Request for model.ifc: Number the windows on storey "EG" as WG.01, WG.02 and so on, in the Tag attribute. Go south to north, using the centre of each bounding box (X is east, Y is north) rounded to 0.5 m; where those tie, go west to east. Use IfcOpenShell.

First a look at what the model holds.

```python
import ifcopenshell
import ifcopenshell.util.element
import ifcopenshell.util.placement

model = ifcopenshell.open("model.ifc")
print(model.schema)
storey = next(s for s in model.by_type("IfcBuildingStorey") if s.Name == "EG")
windows = [e for e in ifcopenshell.util.element.get_decomposition(storey) if e.is_a("IfcWindow")]
for e in sorted(windows, key=lambda e: e.id()):
    origin = ifcopenshell.util.placement.get_local_placement(e.ObjectPlacement)[:3, 3]
    print(e.id(), e.Tag, e.Name, origin.round(2) + 0.0, sep=" | ")
```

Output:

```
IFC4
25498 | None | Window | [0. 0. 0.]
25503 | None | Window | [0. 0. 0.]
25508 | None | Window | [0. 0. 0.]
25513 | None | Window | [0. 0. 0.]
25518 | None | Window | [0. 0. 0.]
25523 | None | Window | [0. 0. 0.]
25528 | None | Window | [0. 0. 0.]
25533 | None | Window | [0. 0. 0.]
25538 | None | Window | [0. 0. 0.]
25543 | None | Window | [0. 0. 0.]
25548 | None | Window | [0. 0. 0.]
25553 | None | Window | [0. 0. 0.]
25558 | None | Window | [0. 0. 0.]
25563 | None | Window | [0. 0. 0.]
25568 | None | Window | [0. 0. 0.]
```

```python
import ifcopenshell
import ifcopenshell.geom
import ifcopenshell.util.element
import ifcopenshell.util.shape

model = ifcopenshell.open("model.ifc")
settings = ifcopenshell.geom.settings()
settings.set("use-world-coords", True)


def centre(element):
    shape = ifcopenshell.geom.create_shape(settings, element)
    return ifcopenshell.util.shape.get_bbox_centroid(shape.geometry)


storey = next(s for s in model.by_type("IfcBuildingStorey") if s.Name == "EG")
windows = [e for e in ifcopenshell.util.element.get_decomposition(storey) if e.is_a("IfcWindow")]

# Insertion points can sit at a corner or the storey origin, so sort by the geometry (in metres).
centres = {e: centre(e) for e in windows}
windows.sort(key=lambda e: (round(centres[e][1] / 0.5), centres[e][0]))

for i, e in enumerate(windows, start=1):
    number = f"WG.{i:02d}"
    e.Tag = number
    print(e.id(), number)

model.write("model_edited.ifc")
```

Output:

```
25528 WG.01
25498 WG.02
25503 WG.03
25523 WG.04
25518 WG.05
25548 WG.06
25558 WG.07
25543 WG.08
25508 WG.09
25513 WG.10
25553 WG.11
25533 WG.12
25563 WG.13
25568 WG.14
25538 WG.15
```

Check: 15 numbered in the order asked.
